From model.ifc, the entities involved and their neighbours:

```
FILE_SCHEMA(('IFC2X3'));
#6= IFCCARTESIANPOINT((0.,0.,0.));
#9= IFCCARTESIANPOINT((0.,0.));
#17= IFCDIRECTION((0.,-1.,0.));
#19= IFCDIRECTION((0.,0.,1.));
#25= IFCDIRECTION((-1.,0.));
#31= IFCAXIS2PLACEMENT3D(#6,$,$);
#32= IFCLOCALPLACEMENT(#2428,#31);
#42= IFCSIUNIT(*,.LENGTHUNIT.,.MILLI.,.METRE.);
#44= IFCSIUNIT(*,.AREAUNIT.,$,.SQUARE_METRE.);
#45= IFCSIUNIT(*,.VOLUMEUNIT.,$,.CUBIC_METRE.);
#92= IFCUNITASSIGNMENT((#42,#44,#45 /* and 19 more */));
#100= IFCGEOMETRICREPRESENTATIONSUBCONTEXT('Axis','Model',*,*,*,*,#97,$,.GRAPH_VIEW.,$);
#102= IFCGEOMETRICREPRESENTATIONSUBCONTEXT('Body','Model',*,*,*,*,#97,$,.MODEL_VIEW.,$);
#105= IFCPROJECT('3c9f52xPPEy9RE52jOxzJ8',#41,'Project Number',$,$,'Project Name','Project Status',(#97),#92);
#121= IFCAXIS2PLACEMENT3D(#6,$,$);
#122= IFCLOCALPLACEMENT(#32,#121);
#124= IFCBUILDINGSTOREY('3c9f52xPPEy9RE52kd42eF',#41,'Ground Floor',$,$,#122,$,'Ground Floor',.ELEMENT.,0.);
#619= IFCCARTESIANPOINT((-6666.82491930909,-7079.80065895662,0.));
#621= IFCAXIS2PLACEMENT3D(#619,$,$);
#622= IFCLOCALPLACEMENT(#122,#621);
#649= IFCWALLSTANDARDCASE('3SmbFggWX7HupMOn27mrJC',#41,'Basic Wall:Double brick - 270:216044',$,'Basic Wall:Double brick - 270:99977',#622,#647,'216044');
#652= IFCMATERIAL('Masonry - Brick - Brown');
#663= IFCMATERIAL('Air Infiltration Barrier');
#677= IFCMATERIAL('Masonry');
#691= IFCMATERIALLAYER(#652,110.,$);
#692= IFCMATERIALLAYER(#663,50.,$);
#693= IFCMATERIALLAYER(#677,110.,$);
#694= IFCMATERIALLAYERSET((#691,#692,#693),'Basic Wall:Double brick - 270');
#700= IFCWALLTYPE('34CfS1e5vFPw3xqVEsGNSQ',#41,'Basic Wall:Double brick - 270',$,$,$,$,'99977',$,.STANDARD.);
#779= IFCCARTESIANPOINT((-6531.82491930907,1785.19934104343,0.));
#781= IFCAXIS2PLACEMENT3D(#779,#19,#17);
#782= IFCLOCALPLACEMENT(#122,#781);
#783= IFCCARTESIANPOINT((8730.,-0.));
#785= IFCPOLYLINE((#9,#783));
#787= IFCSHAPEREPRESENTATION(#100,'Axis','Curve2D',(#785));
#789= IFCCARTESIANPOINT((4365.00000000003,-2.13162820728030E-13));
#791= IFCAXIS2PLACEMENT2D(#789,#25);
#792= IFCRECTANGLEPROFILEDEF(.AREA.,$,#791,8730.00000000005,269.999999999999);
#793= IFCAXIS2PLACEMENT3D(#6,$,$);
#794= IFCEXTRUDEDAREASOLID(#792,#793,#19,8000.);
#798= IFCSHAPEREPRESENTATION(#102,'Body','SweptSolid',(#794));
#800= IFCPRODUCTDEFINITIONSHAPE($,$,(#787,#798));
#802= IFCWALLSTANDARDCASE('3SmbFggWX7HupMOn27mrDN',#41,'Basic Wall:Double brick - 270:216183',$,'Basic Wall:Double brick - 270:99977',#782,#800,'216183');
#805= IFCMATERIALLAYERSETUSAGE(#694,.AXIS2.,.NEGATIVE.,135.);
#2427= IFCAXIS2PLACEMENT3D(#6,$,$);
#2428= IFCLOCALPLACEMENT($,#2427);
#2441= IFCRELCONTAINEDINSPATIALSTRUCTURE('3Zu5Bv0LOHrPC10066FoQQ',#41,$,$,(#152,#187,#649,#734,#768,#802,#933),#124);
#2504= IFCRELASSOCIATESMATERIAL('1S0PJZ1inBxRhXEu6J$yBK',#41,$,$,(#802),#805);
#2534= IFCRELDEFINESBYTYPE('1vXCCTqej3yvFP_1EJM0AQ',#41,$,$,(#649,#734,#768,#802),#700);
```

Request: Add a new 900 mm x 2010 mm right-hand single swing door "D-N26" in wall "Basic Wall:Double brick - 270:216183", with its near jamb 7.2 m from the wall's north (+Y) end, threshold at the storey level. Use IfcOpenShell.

```python
import numpy as np
import ifcopenshell
import ifcopenshell.api.feature
import ifcopenshell.api.geometry
import ifcopenshell.api.root
import ifcopenshell.api.spatial
import ifcopenshell.api.type
import ifcopenshell.geom
import ifcopenshell.util.element
import ifcopenshell.util.placement
import ifcopenshell.util.representation
import ifcopenshell.util.shape
import ifcopenshell.util.unit

model = ifcopenshell.open("model.ifc")
unit_scale = ifcopenshell.util.unit.calculate_unit_scale(model)
settings = ifcopenshell.geom.settings()


def volume(element):
    """Net volume in cubic metres, openings subtracted."""
    shape = ifcopenshell.geom.create_shape(settings, element)
    return ifcopenshell.util.shape.get_volume(shape.geometry)


wall = model.by_guid("3SmbFggWX7HupMOn27mrDN")
storey = ifcopenshell.util.element.get_container(wall, ifc_class="IfcBuildingStorey")
context = ifcopenshell.util.representation.get_context(model, "Model", "Body", "MODEL_VIEW")
before = volume(wall)

width, height, from_end, sill = 0.9, 2.01, 7.2, 0.0  # metres

# The wall runs along its own X axis, and the end named is its -X end.
wall_shape = ifcopenshell.geom.create_shape(settings, wall)
x, y, z = ifcopenshell.util.shape.get_vertices(wall_shape.geometry).T
start = x.min() + from_end
face, thickness = float(y.min()), float(y.max() - y.min())
wall_matrix = ifcopenshell.util.placement.get_local_placement(wall.ObjectPlacement)
level = ifcopenshell.util.placement.get_local_placement(storey.ObjectPlacement)[2, 3]


def in_wall(x, y):
    """Placement at x, y metres in the wall's axes, at sill height."""
    matrix = wall_matrix.copy()
    matrix[:, 3] = wall_matrix @ np.array([x / unit_scale, y / unit_scale, 0.0, 1.0])
    matrix[2, 3] = level + sill / unit_scale
    return matrix


# Opening: a box that overshoots both wall faces by 50 mm.
opening = ifcopenshell.api.root.create_entity(model, ifc_class="IfcOpeningElement")
box = ifcopenshell.api.geometry.add_wall_representation(
    model, context=context, length=width, height=height, thickness=thickness + 0.1
)
ifcopenshell.api.geometry.assign_representation(model, product=opening, representation=box)
ifcopenshell.api.geometry.edit_object_placement(model, product=opening, matrix=in_wall(start, face - 0.05), is_si=False)
ifcopenshell.api.feature.add_feature(model, feature=opening, element=wall)

door = ifcopenshell.api.root.create_entity(model, ifc_class="IfcDoor", name="D-N26")
door.OverallWidth, door.OverallHeight = width / unit_scale, height / unit_scale
body = ifcopenshell.api.geometry.add_door_representation(
    model,
    context=context,
    overall_width=door.OverallWidth,
    overall_height=door.OverallHeight,
    operation_type="SINGLE_SWING_RIGHT",
    lining_properties={"LiningDepth": thickness / unit_scale, "ThresholdDepth": thickness / unit_scale},
)
ifcopenshell.api.geometry.assign_representation(model, product=door, representation=body)
ifcopenshell.api.spatial.assign_container(model, products=[door], relating_structure=storey)
fills = ifcopenshell.api.feature.add_filling(model, opening=opening, element=door)
fills.OwnerHistory = door.OwnerHistory  # required in IFC2X3

# IFC2X3 keeps the operation on the door style.
style = ifcopenshell.api.root.create_entity(model, ifc_class="IfcDoorStyle", name="D-N26")
style.OperationType, style.ConstructionType = "SINGLE_SWING_RIGHT", "NOTDEFINED"
style.ParameterTakesPrecedence = style.Sizeable = False
ifcopenshell.api.type.assign_type(model, related_objects=[door], relating_type=style)

# The lining spans the wall, so the door starts at the wall face.
ifcopenshell.api.geometry.edit_object_placement(model, product=door, matrix=in_wall(start, face), is_si=False)

after = volume(wall)

print(f"wall volume {before:.3f} -> {after:.3f} m3")

model.write("model_edited.ifc")
```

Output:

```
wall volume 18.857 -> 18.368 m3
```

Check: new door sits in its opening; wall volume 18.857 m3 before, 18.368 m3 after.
